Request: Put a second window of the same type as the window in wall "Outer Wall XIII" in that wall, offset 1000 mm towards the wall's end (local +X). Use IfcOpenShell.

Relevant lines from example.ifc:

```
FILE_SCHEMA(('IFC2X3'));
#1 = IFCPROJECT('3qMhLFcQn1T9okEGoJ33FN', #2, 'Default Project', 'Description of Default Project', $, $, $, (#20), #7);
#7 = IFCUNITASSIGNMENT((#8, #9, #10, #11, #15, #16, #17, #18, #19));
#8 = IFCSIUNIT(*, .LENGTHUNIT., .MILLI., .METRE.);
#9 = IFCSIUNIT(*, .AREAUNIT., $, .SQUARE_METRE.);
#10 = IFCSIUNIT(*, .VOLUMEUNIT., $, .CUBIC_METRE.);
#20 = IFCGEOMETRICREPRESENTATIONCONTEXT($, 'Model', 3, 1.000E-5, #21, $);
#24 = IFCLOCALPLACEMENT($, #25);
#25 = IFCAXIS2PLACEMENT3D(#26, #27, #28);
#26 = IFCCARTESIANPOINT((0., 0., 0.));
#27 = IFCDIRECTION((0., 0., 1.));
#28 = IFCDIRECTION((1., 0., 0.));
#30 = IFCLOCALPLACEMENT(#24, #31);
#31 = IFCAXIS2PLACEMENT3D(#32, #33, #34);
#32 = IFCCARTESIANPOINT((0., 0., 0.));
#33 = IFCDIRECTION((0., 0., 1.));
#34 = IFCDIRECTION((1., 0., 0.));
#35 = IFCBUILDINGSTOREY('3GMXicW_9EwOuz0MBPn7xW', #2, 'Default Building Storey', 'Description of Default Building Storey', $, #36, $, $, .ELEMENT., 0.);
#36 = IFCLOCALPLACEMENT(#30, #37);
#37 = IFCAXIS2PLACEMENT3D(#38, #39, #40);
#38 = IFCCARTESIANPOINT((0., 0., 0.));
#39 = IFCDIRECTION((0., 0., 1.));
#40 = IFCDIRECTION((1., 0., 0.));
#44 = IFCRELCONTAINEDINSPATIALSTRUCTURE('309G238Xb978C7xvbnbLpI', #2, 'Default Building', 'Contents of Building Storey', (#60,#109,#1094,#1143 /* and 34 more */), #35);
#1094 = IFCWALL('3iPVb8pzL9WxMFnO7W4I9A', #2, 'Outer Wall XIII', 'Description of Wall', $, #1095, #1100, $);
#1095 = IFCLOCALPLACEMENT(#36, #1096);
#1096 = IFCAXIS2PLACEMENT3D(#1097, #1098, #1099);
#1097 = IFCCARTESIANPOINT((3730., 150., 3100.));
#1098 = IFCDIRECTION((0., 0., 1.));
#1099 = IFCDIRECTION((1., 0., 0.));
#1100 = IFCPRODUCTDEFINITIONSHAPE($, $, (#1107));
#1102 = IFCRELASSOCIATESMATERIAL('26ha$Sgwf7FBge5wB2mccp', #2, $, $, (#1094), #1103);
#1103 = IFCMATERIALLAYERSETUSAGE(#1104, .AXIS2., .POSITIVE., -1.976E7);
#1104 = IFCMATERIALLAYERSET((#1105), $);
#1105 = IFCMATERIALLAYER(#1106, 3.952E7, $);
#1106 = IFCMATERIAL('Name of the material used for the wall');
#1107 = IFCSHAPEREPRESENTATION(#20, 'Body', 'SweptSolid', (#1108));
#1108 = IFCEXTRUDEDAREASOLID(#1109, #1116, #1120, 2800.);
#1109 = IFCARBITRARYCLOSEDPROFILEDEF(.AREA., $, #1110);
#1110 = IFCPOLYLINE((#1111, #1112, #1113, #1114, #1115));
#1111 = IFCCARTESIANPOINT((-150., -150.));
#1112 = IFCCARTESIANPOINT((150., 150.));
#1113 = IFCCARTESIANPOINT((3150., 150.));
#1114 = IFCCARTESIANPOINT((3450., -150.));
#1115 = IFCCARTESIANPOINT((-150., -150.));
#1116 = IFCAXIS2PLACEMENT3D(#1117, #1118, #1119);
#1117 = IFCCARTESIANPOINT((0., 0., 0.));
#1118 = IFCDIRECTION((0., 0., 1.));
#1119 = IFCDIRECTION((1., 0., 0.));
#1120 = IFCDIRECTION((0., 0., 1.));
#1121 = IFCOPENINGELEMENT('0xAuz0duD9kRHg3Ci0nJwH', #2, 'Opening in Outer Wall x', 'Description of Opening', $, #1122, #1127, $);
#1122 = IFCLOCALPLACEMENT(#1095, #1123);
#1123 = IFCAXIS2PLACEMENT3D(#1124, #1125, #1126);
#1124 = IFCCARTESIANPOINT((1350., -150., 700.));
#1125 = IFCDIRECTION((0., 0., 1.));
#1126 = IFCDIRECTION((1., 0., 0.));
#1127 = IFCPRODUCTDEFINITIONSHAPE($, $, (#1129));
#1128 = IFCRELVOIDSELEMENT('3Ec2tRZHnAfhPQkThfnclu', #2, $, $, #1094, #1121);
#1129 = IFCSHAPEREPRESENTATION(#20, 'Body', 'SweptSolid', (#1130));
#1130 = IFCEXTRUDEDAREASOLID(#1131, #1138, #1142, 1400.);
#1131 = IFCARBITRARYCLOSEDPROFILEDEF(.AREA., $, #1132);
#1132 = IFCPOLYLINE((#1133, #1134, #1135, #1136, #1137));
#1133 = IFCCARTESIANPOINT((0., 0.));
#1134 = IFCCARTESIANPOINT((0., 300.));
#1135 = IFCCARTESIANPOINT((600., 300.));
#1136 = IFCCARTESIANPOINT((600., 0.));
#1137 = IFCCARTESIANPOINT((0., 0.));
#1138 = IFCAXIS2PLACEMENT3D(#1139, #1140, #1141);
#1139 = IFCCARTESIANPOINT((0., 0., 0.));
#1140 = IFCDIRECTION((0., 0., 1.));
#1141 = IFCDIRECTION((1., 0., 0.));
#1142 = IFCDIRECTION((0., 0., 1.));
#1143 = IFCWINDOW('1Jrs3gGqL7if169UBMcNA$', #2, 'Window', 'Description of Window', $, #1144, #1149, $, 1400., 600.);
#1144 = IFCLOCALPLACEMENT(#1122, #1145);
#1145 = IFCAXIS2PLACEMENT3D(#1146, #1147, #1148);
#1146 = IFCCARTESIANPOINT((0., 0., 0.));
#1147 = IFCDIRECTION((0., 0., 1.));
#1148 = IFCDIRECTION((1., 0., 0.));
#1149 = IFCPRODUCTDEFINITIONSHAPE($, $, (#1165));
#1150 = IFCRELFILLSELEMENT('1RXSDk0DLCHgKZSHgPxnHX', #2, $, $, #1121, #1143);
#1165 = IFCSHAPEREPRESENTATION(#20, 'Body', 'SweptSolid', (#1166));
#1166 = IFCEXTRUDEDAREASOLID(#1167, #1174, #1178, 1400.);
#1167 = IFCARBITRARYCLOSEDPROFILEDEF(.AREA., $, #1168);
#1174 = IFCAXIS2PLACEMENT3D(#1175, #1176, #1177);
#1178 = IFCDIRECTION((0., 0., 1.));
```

```python
import ifcopenshell
import ifcopenshell.api.feature
import ifcopenshell.api.geometry
import ifcopenshell.api.root
import ifcopenshell.geom
import ifcopenshell.util.element
import ifcopenshell.util.placement
import ifcopenshell.util.shape

model = ifcopenshell.open("example.ifc")
settings = ifcopenshell.geom.settings()


def volume(element):
    """Net volume in cubic metres, openings subtracted."""
    shape = ifcopenshell.geom.create_shape(settings, element)
    return ifcopenshell.util.shape.get_volume(shape.geometry)


def reuse_history(source, copy):
    """copy_class also copies each property set's owner history, people and application; keep the originals."""
    for rel in copy.IsDefinedBy:
        if rel.is_a("IfcRelDefinesByProperties") and (history := rel.RelatingPropertyDefinition.OwnerHistory):
            rel.RelatingPropertyDefinition.OwnerHistory = source.OwnerHistory
            ifcopenshell.util.element.remove_deep2(model, history)


window = model.by_id(1143)
opening = window.FillsVoids[0].RelatingOpeningElement
wall = opening.VoidsElements[0].RelatingBuildingElement
before = volume(wall)
shift = ifcopenshell.util.placement.get_local_placement(wall.ObjectPlacement)[:3, 0] * 1000.0

# copy_class copies the void relationship, type, container and properties, but no geometry.
new_opening = ifcopenshell.api.root.copy_class(model, product=opening)
new_opening.Representation = ifcopenshell.util.element.copy_deep(
    model, opening.Representation, exclude=["IfcGeometricRepresentationContext", "IfcRepresentationMap"]
)
new_window = ifcopenshell.api.root.copy_class(model, product=window)
new_window.Representation = ifcopenshell.util.element.copy_deep(
    model, window.Representation, exclude=["IfcGeometricRepresentationContext", "IfcRepresentationMap"]
)
reuse_history(window, new_window)
fills = ifcopenshell.api.feature.add_filling(model, opening=new_opening, element=new_window)
fills.OwnerHistory = new_window.OwnerHistory  # required in IFC2X3

for old, new in ((opening, new_opening), (window, new_window)):
    matrix = ifcopenshell.util.placement.get_local_placement(old.ObjectPlacement)
    matrix[:3, 3] += shift
    ifcopenshell.api.geometry.edit_object_placement(model, product=new, matrix=matrix, is_si=False)

after = volume(wall)

print(f"wall volume {before:.3f} -> {after:.3f} m3")

model.write("example_updated.ifc")
```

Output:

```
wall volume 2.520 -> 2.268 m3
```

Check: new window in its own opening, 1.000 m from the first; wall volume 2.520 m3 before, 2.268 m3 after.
